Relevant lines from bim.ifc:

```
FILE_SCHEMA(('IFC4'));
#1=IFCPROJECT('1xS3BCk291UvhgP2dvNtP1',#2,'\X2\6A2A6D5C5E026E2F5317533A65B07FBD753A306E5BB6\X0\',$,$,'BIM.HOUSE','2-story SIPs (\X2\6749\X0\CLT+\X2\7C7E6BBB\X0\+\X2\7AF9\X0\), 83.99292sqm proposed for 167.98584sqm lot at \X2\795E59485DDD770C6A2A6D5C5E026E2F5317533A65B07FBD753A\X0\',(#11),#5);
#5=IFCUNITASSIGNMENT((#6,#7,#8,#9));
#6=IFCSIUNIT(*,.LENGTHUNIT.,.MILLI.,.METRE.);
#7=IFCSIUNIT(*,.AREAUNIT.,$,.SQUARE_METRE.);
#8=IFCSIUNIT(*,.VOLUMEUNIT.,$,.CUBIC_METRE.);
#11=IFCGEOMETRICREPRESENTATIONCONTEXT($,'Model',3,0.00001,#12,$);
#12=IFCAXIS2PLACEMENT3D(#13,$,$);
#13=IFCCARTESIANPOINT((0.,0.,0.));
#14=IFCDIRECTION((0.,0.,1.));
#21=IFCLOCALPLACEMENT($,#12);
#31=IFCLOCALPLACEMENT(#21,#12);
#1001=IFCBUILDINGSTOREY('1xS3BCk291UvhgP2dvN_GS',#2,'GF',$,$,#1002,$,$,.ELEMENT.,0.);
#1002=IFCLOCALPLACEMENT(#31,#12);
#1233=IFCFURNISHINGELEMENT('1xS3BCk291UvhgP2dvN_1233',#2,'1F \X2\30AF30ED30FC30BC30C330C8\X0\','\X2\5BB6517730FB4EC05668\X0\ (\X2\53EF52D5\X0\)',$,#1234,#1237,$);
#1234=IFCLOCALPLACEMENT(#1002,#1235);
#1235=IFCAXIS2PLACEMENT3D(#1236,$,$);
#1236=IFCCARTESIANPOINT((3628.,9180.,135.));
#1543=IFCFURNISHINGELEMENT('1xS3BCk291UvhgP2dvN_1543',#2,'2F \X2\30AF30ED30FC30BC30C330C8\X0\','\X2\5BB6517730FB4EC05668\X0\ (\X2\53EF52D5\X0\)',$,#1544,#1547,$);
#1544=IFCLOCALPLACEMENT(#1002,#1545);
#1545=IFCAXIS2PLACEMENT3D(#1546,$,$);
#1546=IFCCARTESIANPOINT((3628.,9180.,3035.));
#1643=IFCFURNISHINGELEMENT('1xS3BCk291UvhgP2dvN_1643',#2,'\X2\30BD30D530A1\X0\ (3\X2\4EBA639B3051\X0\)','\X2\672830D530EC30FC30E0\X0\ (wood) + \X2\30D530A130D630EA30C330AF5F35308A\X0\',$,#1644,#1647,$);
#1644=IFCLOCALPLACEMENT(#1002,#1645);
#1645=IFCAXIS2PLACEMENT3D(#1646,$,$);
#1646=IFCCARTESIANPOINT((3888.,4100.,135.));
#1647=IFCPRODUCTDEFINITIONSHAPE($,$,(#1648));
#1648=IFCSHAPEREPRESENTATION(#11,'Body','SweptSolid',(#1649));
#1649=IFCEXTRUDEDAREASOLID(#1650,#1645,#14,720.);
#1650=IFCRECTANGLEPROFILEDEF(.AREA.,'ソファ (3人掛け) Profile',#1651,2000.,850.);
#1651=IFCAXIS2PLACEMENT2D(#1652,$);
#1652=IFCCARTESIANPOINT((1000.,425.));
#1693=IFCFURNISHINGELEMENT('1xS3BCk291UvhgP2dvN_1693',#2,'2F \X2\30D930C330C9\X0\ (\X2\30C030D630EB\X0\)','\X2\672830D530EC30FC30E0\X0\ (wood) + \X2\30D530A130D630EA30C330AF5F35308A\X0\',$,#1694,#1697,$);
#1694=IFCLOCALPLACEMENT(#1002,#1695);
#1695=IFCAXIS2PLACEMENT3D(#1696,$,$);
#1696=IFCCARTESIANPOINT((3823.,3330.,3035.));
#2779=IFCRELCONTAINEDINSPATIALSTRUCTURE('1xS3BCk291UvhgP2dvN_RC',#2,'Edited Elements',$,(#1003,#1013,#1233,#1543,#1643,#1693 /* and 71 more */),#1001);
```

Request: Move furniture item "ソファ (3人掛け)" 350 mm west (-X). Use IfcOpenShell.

```python
import ifcopenshell
import ifcopenshell.api.geometry
import ifcopenshell.util.placement

model = ifcopenshell.open("bim.ifc")

item = model.by_id(1643)
matrix = ifcopenshell.util.placement.get_local_placement(item.ObjectPlacement)
matrix[0, 3] -= 350.0
ifcopenshell.api.geometry.edit_object_placement(model, product=item, matrix=matrix, is_si=False)

print(ifcopenshell.util.placement.get_local_placement(item.ObjectPlacement).round(3) + 0.0)

model.write("bim_updated.ifc")
```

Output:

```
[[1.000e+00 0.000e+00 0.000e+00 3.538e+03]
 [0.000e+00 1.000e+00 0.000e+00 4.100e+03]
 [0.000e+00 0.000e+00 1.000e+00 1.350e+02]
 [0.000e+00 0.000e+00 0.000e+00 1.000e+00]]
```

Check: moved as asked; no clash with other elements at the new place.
